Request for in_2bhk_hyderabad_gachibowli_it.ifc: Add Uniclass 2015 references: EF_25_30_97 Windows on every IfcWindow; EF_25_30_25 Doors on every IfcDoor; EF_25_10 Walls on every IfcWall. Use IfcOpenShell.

First a look at what the model holds.

```python
import ifcopenshell

model = ifcopenshell.open("in_2bhk_hyderabad_gachibowli_it.ifc")
print(model.schema)
print("classifications:", [c.Name for c in model.by_type("IfcClassification")])
for ifc_class in ("IfcDoor", "IfcRoof", "IfcStair", "IfcWall", "IfcWindow"):
    print(ifc_class, len(model.by_type(ifc_class)))
```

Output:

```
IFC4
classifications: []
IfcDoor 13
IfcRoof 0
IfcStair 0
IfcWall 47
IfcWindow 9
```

```python
import ifcopenshell
import ifcopenshell.api.classification

model = ifcopenshell.open("in_2bhk_hyderabad_gachibowli_it.ifc")

system = ifcopenshell.api.classification.add_classification(model, classification="Uniclass 2015")

codes = {
    "IfcWindow": ("EF_25_30_97", "Windows"),
    "IfcDoor": ("EF_25_30_25", "Doors"),
    "IfcWall": ("EF_25_10", "Walls"),
}
for ifc_class, (code, name) in codes.items():
    products = model.by_type(ifc_class)
    ifcopenshell.api.classification.add_reference(
        model, products=products, classification=system, identification=code, name=name
    )
    print(code, len(products))

model.write("in_2bhk_hyderabad_gachibowli_it_rev.ifc")
```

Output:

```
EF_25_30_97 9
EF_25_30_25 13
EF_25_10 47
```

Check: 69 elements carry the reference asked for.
